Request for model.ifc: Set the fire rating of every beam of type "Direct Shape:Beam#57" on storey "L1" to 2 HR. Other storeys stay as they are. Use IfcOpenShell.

First a look at what the model holds.

```python
import ifcopenshell
import ifcopenshell.util.element

model = ifcopenshell.open("model.ifc")
print(model.schema)
storey = next(s for s in model.by_type("IfcBuildingStorey") if s.Name == "L1")
beams = [e for e in ifcopenshell.util.element.get_decomposition(storey) if e.is_a("IfcBeam")]
seen = {}
for e in beams:
    element_type = ifcopenshell.util.element.get_type(e)
    key = (element_type.Name if element_type != e and element_type else None, ifcopenshell.util.element.get_pset(e, "Pset_BeamCommon", "FireRating"))
    seen[key] = seen.get(key, 0) + 1
for (name, value), count in sorted(seen.items(), key=str):
    print(count, "x", name, "|", value)
```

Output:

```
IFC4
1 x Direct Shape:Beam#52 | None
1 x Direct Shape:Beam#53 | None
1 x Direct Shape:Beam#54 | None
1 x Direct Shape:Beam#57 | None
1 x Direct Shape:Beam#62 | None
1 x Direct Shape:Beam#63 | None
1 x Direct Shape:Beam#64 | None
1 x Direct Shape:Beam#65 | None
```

```python
import ifcopenshell
import ifcopenshell.api.pset
import ifcopenshell.util.element

model = ifcopenshell.open("model.ifc")

storey = next(s for s in model.by_type("IfcBuildingStorey") if s.Name == "L1")
beams = [e for e in ifcopenshell.util.element.get_decomposition(storey) if e.is_a("IfcBeam")]

count = 0
for e in beams:
    element_type = ifcopenshell.util.element.get_type(e)
    if element_type in (None, e) or element_type.Name != "Direct Shape:Beam#57":
        continue
    # add_pset returns the element's existing set when there is one.
    pset = ifcopenshell.api.pset.add_pset(model, product=e, name="Pset_BeamCommon")
    ifcopenshell.api.pset.edit_pset(model, pset=pset, properties={"FireRating": "2 HR"})
    count += 1

print(count, "beams updated")

model.write("model_rev.ifc")
```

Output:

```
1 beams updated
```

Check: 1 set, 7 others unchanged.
